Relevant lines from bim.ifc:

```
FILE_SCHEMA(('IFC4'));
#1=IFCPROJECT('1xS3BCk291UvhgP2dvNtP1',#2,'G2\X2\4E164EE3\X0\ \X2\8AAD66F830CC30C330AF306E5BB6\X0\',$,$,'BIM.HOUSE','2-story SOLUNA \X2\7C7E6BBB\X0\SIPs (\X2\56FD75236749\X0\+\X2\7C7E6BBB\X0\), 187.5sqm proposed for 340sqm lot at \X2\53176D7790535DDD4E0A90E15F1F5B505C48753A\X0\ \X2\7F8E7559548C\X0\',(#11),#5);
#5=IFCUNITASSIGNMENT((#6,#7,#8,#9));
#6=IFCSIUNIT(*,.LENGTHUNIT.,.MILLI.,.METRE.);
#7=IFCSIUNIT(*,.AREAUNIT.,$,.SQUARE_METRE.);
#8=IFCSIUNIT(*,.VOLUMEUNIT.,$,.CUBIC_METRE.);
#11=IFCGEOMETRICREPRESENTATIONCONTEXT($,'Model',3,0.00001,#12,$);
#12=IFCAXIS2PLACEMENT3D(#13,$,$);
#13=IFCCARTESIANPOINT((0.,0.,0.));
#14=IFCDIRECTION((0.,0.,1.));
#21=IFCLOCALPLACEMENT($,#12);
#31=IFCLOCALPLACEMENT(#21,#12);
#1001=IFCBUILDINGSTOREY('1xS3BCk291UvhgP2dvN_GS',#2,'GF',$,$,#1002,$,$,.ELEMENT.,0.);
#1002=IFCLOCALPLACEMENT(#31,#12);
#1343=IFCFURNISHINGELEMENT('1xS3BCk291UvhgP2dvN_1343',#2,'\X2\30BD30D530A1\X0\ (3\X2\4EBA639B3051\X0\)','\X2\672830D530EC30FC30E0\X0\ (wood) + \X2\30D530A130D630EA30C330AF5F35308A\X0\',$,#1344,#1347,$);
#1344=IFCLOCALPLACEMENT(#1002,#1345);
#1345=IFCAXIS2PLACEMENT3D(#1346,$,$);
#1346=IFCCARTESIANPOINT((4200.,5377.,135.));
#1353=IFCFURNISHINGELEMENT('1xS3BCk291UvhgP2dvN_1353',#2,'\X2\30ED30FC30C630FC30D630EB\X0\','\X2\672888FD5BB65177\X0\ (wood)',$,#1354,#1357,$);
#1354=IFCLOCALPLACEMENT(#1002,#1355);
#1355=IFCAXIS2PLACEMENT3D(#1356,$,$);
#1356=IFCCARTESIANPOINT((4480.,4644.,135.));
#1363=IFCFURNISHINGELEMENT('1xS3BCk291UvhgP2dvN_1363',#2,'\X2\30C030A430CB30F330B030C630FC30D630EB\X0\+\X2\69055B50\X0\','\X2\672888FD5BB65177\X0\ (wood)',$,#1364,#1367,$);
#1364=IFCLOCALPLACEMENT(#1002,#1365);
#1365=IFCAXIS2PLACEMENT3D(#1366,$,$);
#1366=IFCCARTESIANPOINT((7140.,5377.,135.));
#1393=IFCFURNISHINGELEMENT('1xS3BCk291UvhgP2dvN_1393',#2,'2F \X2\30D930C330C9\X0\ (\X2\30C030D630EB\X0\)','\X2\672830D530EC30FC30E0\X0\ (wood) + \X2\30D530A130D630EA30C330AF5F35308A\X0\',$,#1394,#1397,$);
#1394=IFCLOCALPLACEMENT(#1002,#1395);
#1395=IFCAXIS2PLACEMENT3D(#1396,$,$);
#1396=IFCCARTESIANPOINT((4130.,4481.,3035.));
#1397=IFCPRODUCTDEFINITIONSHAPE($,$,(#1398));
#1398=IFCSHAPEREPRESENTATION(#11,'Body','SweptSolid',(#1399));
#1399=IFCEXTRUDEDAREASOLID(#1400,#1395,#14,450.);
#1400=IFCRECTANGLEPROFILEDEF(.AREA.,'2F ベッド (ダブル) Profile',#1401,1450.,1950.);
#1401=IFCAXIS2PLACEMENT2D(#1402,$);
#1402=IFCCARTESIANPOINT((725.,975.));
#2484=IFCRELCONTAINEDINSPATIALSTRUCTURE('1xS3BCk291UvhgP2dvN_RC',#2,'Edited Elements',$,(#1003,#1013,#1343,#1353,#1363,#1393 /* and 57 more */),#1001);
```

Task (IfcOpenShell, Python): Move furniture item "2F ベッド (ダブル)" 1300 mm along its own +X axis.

```python
import ifcopenshell
import ifcopenshell.api.geometry
import ifcopenshell.util.placement

model = ifcopenshell.open("bim.ifc")

item = model.by_id(1393)
matrix = ifcopenshell.util.placement.get_local_placement(item.ObjectPlacement)
matrix[:3, 3] += matrix[:3, 0] * 1300.0
ifcopenshell.api.geometry.edit_object_placement(model, product=item, matrix=matrix, is_si=False)

print(ifcopenshell.util.placement.get_local_placement(item.ObjectPlacement).round(3) + 0.0)

model.write("bim_edited.ifc")
```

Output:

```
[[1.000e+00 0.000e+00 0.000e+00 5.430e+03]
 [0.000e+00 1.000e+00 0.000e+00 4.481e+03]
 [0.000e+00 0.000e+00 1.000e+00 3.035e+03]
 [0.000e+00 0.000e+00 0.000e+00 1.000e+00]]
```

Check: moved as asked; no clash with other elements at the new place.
